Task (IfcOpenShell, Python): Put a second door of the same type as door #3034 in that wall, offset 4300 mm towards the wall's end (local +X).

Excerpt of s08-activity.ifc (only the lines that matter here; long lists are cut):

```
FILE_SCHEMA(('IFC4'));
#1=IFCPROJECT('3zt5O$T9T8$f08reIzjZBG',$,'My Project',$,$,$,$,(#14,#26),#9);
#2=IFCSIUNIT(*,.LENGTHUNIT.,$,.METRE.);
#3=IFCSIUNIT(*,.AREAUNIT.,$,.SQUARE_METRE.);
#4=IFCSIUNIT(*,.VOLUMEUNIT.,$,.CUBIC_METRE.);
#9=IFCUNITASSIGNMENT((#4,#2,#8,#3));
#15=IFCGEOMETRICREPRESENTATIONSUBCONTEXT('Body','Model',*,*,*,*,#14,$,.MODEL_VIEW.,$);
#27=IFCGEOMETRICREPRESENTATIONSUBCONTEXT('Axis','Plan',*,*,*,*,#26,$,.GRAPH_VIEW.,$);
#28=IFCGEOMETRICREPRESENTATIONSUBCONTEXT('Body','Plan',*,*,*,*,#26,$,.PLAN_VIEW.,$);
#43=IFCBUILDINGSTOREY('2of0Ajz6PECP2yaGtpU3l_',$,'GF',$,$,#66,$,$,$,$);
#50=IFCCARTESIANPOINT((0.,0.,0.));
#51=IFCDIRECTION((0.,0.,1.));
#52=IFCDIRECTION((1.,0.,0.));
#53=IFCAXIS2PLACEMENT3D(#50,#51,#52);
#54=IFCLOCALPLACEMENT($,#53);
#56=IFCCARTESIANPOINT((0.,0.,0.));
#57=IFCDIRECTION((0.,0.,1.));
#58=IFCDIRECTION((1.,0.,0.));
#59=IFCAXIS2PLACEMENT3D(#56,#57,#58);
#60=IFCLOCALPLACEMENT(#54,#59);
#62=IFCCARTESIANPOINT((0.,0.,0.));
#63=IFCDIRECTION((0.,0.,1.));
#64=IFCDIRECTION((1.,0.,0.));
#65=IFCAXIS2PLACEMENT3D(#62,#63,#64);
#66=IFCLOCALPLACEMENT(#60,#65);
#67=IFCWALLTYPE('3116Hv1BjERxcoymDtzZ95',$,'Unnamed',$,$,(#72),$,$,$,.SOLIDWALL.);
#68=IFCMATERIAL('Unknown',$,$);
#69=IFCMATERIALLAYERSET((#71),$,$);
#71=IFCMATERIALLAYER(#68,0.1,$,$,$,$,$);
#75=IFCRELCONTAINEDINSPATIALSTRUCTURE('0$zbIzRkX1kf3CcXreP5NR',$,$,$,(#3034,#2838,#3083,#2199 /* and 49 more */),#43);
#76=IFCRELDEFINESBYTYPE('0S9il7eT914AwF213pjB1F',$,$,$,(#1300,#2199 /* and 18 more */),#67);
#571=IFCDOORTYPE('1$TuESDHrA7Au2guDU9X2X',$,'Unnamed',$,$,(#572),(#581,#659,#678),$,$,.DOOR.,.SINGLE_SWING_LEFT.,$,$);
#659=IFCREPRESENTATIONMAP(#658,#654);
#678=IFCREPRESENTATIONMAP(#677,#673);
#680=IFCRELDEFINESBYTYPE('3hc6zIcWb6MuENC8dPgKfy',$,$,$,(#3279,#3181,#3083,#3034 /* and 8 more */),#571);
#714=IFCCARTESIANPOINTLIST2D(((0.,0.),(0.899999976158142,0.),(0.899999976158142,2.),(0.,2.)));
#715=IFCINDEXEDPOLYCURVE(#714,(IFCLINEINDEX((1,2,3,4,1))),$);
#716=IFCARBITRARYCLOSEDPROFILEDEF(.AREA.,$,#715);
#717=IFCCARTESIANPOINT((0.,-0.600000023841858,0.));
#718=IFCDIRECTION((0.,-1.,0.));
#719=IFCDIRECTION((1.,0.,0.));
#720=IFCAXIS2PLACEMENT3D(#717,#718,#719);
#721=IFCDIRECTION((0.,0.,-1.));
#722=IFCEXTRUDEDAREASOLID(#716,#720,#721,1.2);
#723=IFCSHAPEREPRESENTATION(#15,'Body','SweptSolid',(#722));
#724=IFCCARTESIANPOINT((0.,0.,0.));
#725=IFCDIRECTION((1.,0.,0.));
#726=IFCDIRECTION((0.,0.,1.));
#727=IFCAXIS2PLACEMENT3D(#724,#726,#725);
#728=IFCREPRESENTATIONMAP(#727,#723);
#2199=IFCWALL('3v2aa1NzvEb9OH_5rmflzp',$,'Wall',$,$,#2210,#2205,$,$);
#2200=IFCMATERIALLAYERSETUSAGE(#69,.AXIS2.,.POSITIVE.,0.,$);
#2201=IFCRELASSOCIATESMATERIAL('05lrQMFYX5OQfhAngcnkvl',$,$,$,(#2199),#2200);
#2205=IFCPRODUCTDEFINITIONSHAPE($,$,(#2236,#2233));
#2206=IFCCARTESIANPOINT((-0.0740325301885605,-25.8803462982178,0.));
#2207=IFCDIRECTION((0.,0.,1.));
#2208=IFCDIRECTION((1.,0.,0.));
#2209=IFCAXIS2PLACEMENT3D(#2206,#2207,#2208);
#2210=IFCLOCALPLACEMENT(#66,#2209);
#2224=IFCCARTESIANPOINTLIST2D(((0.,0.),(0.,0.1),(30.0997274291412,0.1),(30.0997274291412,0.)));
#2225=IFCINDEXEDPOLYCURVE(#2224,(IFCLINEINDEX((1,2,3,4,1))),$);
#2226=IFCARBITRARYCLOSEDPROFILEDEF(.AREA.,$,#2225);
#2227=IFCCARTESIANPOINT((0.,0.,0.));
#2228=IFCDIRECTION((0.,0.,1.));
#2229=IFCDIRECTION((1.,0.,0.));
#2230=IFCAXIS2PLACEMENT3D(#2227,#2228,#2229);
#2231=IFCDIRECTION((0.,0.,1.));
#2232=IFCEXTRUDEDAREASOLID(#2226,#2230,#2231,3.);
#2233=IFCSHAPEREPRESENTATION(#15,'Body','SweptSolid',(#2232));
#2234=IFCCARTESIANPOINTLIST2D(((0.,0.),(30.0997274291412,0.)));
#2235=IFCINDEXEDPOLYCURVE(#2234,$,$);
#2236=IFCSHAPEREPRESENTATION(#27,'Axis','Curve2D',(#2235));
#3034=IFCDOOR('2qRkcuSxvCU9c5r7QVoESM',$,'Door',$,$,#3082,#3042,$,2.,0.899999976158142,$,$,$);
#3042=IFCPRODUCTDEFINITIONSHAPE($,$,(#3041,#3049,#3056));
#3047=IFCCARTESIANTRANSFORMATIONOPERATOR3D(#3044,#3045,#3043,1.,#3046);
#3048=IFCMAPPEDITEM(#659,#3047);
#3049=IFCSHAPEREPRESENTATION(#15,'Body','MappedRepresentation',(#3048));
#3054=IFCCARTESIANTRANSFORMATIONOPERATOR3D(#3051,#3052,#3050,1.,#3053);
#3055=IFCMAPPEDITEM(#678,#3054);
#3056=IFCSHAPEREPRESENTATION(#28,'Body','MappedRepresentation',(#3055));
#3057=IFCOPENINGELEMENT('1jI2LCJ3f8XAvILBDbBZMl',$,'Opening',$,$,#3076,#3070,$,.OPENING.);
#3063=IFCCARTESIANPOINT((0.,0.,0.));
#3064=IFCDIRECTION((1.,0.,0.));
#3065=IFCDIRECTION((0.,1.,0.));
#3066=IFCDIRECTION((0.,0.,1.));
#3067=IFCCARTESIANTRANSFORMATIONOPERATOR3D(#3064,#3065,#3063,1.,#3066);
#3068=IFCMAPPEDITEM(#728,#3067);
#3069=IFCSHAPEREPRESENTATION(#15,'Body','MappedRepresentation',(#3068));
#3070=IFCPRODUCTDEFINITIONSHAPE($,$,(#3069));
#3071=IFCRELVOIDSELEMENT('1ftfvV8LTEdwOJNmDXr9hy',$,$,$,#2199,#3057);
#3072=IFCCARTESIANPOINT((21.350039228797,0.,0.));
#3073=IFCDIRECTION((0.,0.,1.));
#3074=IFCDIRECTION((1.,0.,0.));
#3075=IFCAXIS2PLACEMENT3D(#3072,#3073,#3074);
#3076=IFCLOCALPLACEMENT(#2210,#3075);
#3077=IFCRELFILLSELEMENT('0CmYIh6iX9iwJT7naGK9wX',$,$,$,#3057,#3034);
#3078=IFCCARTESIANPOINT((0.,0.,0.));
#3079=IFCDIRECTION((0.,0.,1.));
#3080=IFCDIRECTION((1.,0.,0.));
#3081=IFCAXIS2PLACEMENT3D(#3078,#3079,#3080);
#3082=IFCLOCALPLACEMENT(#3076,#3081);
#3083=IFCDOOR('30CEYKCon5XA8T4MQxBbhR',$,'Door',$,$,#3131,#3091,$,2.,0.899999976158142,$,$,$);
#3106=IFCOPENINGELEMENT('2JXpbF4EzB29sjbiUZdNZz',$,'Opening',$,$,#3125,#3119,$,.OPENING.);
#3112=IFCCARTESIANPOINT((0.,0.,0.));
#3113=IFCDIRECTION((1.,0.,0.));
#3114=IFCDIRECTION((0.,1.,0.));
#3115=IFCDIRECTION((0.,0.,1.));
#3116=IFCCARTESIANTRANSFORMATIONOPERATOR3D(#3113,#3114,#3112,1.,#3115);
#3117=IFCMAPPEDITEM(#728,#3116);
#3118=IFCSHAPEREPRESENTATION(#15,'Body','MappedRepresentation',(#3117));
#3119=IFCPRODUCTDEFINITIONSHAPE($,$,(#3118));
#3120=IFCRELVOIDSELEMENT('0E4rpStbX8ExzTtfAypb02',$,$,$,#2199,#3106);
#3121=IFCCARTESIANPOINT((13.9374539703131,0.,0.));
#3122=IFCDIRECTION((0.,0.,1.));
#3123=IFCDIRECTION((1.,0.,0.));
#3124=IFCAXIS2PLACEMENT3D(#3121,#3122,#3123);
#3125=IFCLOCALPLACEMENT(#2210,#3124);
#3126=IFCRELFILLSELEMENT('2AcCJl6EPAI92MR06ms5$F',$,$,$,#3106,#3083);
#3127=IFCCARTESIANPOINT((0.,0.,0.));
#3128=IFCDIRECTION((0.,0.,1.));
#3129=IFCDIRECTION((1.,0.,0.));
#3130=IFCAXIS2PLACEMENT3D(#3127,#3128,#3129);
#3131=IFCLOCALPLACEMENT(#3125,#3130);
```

```python
import ifcopenshell
import ifcopenshell.api.feature
import ifcopenshell.api.geometry
import ifcopenshell.api.root
import ifcopenshell.geom
import ifcopenshell.util.element
import ifcopenshell.util.placement
import ifcopenshell.util.shape

model = ifcopenshell.open("s08-activity.ifc")
settings = ifcopenshell.geom.settings()


def volume(element):
    """Net volume in cubic metres, openings subtracted."""
    shape = ifcopenshell.geom.create_shape(settings, element)
    return ifcopenshell.util.shape.get_volume(shape.geometry)


door = model.by_guid("2qRkcuSxvCU9c5r7QVoESM")
opening = door.FillsVoids[0].RelatingOpeningElement
wall = opening.VoidsElements[0].RelatingBuildingElement
before = volume(wall)
shift = ifcopenshell.util.placement.get_local_placement(wall.ObjectPlacement)[:3, 0] * 4.3

# copy_class copies the void relationship, type, container and properties, but no geometry.
new_opening = ifcopenshell.api.root.copy_class(model, product=opening)
new_opening.Representation = ifcopenshell.util.element.copy_deep(
    model, opening.Representation, exclude=["IfcGeometricRepresentationContext", "IfcRepresentationMap"]
)
new_door = ifcopenshell.api.root.copy_class(model, product=door)
new_door.Representation = ifcopenshell.util.element.copy_deep(
    model, door.Representation, exclude=["IfcGeometricRepresentationContext", "IfcRepresentationMap"]
)
ifcopenshell.api.feature.add_filling(model, opening=new_opening, element=new_door)

for old, new in ((opening, new_opening), (door, new_door)):
    matrix = ifcopenshell.util.placement.get_local_placement(old.ObjectPlacement)
    matrix[:3, 3] += shift
    ifcopenshell.api.geometry.edit_object_placement(model, product=new, matrix=matrix, is_si=False)

after = volume(wall)

print(f"wall volume {before:.3f} -> {after:.3f} m3")

model.write("s08-activity-out.ifc")
```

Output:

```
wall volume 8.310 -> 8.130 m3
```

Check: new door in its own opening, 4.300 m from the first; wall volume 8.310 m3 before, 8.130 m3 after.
